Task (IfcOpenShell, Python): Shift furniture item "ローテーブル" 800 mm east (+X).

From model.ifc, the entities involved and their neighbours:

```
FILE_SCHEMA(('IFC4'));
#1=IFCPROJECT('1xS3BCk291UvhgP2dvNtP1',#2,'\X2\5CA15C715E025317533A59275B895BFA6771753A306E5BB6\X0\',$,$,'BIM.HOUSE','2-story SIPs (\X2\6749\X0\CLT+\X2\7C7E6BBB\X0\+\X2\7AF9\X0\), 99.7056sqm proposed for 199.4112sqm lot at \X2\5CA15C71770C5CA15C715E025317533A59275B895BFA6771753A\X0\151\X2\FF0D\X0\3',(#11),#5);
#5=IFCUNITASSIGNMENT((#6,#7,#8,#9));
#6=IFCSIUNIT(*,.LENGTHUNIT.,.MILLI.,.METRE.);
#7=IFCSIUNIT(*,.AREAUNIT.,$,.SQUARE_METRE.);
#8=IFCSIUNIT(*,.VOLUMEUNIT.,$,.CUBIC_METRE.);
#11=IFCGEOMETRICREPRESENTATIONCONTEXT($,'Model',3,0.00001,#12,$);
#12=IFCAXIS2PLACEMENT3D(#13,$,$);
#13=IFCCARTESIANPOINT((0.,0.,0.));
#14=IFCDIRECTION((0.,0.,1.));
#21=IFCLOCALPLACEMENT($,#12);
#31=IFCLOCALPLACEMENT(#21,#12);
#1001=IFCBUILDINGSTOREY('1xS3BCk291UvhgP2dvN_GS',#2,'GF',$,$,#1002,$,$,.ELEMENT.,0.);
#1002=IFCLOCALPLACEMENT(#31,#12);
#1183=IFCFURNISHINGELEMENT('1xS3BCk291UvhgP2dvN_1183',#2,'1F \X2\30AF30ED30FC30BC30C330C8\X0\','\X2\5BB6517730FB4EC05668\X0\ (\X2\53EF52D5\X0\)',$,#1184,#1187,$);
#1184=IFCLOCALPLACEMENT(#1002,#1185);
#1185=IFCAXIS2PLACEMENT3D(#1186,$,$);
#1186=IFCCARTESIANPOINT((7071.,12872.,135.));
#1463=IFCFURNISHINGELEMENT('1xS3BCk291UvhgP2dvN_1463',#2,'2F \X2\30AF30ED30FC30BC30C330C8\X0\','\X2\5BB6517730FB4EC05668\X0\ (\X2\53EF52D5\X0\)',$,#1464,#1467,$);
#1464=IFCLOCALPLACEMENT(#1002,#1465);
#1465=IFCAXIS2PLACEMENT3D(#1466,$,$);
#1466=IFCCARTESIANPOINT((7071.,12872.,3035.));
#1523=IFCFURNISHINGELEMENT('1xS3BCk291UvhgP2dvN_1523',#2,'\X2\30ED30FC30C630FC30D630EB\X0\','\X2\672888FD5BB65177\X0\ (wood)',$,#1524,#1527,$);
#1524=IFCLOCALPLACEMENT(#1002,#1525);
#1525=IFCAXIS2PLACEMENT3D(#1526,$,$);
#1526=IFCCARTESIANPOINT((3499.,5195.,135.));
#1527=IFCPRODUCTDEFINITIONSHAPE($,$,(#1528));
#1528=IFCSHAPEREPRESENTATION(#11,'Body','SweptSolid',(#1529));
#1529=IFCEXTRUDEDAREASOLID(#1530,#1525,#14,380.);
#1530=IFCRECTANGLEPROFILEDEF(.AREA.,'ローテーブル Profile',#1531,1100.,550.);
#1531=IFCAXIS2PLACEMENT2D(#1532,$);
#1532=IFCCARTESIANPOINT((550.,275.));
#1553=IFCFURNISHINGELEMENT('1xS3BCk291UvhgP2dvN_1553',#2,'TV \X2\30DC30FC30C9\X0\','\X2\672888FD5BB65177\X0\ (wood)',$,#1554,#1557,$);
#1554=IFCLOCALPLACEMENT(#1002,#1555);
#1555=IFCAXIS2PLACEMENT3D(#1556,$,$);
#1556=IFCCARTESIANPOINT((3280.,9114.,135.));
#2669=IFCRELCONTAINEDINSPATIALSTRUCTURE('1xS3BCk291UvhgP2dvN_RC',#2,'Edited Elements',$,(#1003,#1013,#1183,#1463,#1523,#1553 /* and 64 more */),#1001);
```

```python
import ifcopenshell
import ifcopenshell.api.geometry
import ifcopenshell.util.placement
import ifcopenshell.util.unit

model = ifcopenshell.open("model.ifc")
unit_scale = ifcopenshell.util.unit.calculate_unit_scale(model)

item = model.by_id(1523)
matrix = ifcopenshell.util.placement.get_local_placement(item.ObjectPlacement)
matrix[0, 3] += 0.8 / unit_scale
ifcopenshell.api.geometry.edit_object_placement(model, product=item, matrix=matrix, is_si=False)

print(ifcopenshell.util.placement.get_local_placement(item.ObjectPlacement).round(3) + 0.0)

model.write("model_edited.ifc")
```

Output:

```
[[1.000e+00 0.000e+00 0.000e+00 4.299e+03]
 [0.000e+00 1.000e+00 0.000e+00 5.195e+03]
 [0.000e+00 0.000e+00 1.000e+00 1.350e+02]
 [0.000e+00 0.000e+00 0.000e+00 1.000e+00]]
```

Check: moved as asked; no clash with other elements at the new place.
